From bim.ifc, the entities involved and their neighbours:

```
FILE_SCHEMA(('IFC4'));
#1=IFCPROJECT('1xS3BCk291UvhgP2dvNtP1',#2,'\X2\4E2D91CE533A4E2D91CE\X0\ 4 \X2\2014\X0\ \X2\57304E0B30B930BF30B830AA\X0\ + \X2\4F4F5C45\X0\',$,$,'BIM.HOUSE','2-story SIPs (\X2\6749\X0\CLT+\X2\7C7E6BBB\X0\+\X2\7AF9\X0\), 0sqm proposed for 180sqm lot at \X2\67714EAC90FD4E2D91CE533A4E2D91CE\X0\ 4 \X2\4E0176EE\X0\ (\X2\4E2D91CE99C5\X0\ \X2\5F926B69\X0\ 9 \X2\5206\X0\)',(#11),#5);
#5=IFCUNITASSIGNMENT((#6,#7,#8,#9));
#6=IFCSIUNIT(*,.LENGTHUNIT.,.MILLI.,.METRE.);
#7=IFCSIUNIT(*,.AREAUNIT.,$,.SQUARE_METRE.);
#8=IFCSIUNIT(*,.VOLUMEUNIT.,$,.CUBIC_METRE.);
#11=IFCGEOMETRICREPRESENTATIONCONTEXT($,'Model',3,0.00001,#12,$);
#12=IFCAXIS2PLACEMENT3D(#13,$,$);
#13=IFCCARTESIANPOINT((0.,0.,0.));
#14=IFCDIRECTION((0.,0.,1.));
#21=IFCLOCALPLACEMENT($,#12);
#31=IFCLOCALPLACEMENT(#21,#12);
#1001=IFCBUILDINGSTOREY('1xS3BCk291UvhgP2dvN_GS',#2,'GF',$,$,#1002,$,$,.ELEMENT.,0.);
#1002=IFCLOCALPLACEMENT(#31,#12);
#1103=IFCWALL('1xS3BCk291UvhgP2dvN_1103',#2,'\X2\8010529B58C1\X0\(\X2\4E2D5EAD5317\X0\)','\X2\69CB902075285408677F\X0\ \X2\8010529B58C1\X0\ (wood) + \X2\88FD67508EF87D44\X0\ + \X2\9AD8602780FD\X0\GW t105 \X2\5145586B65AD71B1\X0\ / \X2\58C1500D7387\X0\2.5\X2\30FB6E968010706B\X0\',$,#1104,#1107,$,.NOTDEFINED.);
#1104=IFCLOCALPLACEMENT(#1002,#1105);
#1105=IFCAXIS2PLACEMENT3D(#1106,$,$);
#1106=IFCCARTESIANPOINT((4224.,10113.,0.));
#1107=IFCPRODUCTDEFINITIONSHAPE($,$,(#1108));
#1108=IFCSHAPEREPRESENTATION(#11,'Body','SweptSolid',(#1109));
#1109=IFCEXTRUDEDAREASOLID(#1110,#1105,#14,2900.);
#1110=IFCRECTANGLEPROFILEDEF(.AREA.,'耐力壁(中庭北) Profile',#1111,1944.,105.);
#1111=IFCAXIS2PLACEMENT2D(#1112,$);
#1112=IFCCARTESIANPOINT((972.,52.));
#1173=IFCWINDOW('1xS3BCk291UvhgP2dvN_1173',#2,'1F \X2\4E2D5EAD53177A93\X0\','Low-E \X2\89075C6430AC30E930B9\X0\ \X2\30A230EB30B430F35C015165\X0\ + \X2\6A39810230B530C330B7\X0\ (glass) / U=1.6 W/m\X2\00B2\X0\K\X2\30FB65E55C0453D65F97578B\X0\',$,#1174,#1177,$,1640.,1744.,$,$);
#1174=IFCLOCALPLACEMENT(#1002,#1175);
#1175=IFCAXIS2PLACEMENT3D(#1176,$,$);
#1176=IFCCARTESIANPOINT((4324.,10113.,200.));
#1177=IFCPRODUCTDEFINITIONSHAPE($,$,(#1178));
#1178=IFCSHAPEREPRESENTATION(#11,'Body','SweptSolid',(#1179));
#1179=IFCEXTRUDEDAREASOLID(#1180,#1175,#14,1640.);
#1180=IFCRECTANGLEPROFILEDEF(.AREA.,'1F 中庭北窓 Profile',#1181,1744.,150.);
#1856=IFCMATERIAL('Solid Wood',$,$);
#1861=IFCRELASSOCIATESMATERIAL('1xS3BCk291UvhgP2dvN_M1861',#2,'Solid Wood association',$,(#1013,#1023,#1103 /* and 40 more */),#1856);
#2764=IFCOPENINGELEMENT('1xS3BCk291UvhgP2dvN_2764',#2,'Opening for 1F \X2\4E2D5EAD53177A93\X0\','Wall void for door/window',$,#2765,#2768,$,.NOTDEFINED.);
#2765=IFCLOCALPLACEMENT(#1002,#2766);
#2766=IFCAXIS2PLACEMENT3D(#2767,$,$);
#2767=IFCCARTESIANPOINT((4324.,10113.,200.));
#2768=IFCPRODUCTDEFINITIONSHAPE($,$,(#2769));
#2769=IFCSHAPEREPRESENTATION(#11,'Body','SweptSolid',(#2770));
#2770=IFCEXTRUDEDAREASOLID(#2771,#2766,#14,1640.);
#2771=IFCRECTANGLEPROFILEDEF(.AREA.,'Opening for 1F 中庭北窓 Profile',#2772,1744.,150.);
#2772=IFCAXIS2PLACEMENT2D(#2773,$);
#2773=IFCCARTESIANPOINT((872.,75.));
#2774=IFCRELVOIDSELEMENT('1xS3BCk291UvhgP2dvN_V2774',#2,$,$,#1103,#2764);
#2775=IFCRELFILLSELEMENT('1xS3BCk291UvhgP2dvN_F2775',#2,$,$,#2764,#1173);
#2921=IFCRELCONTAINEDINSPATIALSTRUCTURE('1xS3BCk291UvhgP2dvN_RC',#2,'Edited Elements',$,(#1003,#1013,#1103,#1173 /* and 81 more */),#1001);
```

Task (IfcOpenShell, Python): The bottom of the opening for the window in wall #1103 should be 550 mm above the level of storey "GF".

```python
import numpy as np
import ifcopenshell
import ifcopenshell.api.geometry
import ifcopenshell.geom
import ifcopenshell.util.element
import ifcopenshell.util.placement
import ifcopenshell.util.shape
import ifcopenshell.util.unit

model = ifcopenshell.open("bim.ifc")
unit_scale = ifcopenshell.util.unit.calculate_unit_scale(model)

window = model.by_id(1173)
opening = window.FillsVoids[0].RelatingOpeningElement
storey = ifcopenshell.util.element.get_container(window, ifc_class="IfcBuildingStorey")
level = ifcopenshell.util.placement.get_local_placement(storey.ObjectPlacement)[2, 3]

# The opening's origin need not be at the sill, so measure its lowest point.
shape = ifcopenshell.geom.create_shape(ifcopenshell.geom.settings(), opening)
bottom = ifcopenshell.util.shape.get_shape_bottom_elevation(shape, shape.geometry) / unit_scale
dz = level + 550.0 - bottom

shift = np.array([0.0, 0.0, dz])
# The window is not placed relative to its opening, so move both.
for product in (opening, window):
    matrix = ifcopenshell.util.placement.get_local_placement(product.ObjectPlacement)
    matrix[:3, 3] += shift
    ifcopenshell.api.geometry.edit_object_placement(model, product=product, matrix=matrix, is_si=False)

print(f"moved by {dz * unit_scale:+.3f} m")

model.write("bim_rev.ifc")
```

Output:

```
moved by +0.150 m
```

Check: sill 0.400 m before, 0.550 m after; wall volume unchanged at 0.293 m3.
